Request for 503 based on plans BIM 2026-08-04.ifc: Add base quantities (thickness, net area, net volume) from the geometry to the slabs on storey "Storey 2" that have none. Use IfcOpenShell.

First a look at what the model holds.

```python
import ifcopenshell
import ifcopenshell.util.element
import ifcopenshell.util.unit

model = ifcopenshell.open("503 based on plans BIM 2026-08-04.ifc")
print(model.schema)
for unit_type in ("LENGTHUNIT", "AREAUNIT", "VOLUMEUNIT"):
    print(unit_type, ifcopenshell.util.unit.calculate_unit_scale(model, unit_type))
storey = next(s for s in model.by_type("IfcBuildingStorey") if s.Name == "Storey 2")
slabs = [e for e in ifcopenshell.util.element.get_decomposition(storey) if e.is_a("IfcSlab")]
for e in sorted(slabs, key=lambda e: e.id()):
    print(e.id(), e.is_a(), e.Name, list(ifcopenshell.util.element.get_psets(e, qtos_only=True)), sep=" | ")
```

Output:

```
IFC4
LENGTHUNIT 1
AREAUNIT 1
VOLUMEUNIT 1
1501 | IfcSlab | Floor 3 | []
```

```python
import ifcopenshell
import ifcopenshell.api.pset
import ifcopenshell.geom
import ifcopenshell.util.element
import ifcopenshell.util.shape
import ifcopenshell.util.unit

model = ifcopenshell.open("503 based on plans BIM 2026-08-04.ifc")
unit_scale = ifcopenshell.util.unit.calculate_unit_scale(model)
area_scale = ifcopenshell.util.unit.calculate_unit_scale(model, "AREAUNIT")
volume_scale = ifcopenshell.util.unit.calculate_unit_scale(model, "VOLUMEUNIT")
settings = ifcopenshell.geom.settings()

storey = next(s for s in model.by_type("IfcBuildingStorey") if s.Name == "Storey 2")
slabs = [e for e in ifcopenshell.util.element.get_decomposition(storey) if e.is_a("IfcSlab")]

for e in sorted(slabs, key=lambda e: e.id()):
    if ifcopenshell.util.element.get_psets(e, qtos_only=True, should_inherit=False):
        continue
    # Geometry comes back in metres, in the element's own axes.
    shape = ifcopenshell.geom.create_shape(settings, e)
    values = {
        "Width": ifcopenshell.util.shape.get_z(shape.geometry) / unit_scale,
        "NetArea": ifcopenshell.util.shape.get_footprint_area(shape.geometry) / area_scale,
        "NetVolume": ifcopenshell.util.shape.get_volume(shape.geometry) / volume_scale,
    }
    qto = ifcopenshell.api.pset.add_qto(model, product=e, name="Qto_SlabBaseQuantities")
    ifcopenshell.api.pset.edit_qto(model, qto=qto, properties=values)
    print(e.id(), {k: round(v, 3) for k, v in values.items()})

model.write("503 based on plans BIM 2026-08-04_rev.ifc")
```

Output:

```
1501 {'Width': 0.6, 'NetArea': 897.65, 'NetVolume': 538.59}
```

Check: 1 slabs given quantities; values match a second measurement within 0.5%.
